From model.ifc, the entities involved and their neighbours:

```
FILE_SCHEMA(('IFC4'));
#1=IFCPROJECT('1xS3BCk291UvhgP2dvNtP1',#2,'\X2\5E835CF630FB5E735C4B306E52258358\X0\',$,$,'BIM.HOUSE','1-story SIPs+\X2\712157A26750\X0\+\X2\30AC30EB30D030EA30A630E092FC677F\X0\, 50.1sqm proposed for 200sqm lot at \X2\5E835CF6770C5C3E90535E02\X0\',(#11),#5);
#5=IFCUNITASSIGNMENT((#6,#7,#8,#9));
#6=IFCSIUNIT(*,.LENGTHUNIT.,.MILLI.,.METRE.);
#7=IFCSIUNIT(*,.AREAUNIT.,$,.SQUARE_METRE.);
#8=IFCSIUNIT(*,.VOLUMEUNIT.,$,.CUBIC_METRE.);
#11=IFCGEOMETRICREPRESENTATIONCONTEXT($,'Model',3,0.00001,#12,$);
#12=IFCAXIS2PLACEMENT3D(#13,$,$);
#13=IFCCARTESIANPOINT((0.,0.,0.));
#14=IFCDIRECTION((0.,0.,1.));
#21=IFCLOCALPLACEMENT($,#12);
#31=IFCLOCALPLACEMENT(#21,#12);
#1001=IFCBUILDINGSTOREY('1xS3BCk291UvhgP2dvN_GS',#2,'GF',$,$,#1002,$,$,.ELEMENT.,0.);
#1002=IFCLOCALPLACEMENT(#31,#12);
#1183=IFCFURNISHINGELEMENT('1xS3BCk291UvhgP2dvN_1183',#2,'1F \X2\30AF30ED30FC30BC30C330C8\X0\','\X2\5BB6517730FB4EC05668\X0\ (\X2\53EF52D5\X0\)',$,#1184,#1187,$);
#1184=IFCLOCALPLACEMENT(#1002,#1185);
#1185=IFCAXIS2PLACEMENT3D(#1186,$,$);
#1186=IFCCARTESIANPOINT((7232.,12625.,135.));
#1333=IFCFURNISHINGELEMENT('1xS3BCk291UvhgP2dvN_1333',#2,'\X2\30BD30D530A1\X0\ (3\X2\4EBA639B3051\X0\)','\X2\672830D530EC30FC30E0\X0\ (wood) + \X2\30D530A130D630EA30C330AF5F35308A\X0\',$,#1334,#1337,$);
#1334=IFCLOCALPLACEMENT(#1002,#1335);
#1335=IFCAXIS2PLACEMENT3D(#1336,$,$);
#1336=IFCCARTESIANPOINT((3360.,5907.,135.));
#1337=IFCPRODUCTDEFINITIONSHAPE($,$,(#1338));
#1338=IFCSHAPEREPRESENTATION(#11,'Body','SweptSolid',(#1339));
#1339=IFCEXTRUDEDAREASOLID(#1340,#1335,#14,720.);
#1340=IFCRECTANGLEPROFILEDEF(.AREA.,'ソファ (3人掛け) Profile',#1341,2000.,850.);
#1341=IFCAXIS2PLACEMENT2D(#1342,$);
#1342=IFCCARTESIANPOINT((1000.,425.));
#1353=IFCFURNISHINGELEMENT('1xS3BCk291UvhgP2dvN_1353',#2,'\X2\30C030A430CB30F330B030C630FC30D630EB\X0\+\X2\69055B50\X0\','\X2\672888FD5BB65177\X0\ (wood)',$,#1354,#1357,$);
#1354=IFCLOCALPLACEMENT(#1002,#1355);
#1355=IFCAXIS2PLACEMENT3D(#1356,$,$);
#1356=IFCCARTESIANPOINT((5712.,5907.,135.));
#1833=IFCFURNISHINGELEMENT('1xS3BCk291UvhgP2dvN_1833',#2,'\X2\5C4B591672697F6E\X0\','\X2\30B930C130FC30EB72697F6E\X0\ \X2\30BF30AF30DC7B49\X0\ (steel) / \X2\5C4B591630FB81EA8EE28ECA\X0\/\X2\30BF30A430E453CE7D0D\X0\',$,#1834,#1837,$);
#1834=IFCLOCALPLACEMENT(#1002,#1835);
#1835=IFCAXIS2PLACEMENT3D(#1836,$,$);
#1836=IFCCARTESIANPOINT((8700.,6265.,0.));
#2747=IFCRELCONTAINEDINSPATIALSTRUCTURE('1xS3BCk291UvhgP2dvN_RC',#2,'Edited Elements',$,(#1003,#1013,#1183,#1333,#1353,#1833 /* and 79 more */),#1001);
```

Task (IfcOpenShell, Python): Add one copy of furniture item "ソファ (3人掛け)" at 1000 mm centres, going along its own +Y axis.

```python
import ifcopenshell
import ifcopenshell.api.geometry
import ifcopenshell.api.root
import ifcopenshell.util.element
import ifcopenshell.util.placement

model = ifcopenshell.open("model.ifc")


def reuse_history(source, copy):
    """copy_class also copies each property set's owner history, people and application; keep the originals."""
    for rel in copy.IsDefinedBy:
        if rel.is_a("IfcRelDefinesByProperties") and (history := rel.RelatingPropertyDefinition.OwnerHistory):
            rel.RelatingPropertyDefinition.OwnerHistory = source.OwnerHistory
            ifcopenshell.util.element.remove_deep2(model, history)


source = model.by_guid("1xS3BCk291UvhgP2dvN_1333")
base = ifcopenshell.util.placement.get_local_placement(source.ObjectPlacement)
step = base[:3, 1] * 1000.0

for i in range(1, 2):
    copy = ifcopenshell.api.root.copy_class(model, product=source)
    copy.Representation = ifcopenshell.util.element.copy_deep(
        model, source.Representation, exclude=["IfcGeometricRepresentationContext", "IfcRepresentationMap"]
    )
    reuse_history(source, copy)
    matrix = base.copy()
    matrix[:3, 3] += i * step
    print("added at", matrix[:3, 3].round(3) + 0.0)
    ifcopenshell.api.geometry.edit_object_placement(model, product=copy, matrix=matrix, is_si=False)

model.write("model_v2.ifc")
```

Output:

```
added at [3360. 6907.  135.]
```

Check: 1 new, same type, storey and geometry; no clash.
